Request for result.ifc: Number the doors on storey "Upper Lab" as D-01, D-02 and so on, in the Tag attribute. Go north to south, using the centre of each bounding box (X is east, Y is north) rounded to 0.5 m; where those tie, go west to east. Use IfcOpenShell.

First a look at what the model holds.

```python
import ifcopenshell
import ifcopenshell.util.element
import ifcopenshell.util.placement

model = ifcopenshell.open("result.ifc")
print(model.schema)
storey = next(s for s in model.by_type("IfcBuildingStorey") if s.Name == "Upper Lab")
doors = [e for e in ifcopenshell.util.element.get_decomposition(storey) if e.is_a("IfcDoor")]
for e in sorted(doors, key=lambda e: e.id()):
    origin = ifcopenshell.util.placement.get_local_placement(e.ObjectPlacement)[:3, 3]
    print(e.id(), e.Tag, e.Name, origin.round(2) + 0.0, sep=" | ")
```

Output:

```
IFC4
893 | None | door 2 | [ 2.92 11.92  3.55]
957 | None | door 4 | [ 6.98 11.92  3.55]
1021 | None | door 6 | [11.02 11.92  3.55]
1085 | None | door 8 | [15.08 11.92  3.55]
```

```python
import ifcopenshell
import ifcopenshell.geom
import ifcopenshell.util.element
import ifcopenshell.util.shape

model = ifcopenshell.open("result.ifc")
settings = ifcopenshell.geom.settings()
settings.set("use-world-coords", True)


def centre(element):
    shape = ifcopenshell.geom.create_shape(settings, element)
    return ifcopenshell.util.shape.get_bbox_centroid(shape.geometry)


storey = next(s for s in model.by_type("IfcBuildingStorey") if s.Name == "Upper Lab")
doors = [e for e in ifcopenshell.util.element.get_decomposition(storey) if e.is_a("IfcDoor")]

# Insertion points can sit at a corner or the storey origin, so sort by the geometry (in metres).
centres = {e: centre(e) for e in doors}
doors.sort(key=lambda e: (-round(centres[e][1] / 0.5), centres[e][0]))

for i, e in enumerate(doors, start=1):
    number = f"D-{i:02d}"
    e.Tag = number
    print(e.id(), number)

model.write("result_edited.ifc")
```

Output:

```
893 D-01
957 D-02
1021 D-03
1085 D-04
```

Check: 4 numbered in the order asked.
